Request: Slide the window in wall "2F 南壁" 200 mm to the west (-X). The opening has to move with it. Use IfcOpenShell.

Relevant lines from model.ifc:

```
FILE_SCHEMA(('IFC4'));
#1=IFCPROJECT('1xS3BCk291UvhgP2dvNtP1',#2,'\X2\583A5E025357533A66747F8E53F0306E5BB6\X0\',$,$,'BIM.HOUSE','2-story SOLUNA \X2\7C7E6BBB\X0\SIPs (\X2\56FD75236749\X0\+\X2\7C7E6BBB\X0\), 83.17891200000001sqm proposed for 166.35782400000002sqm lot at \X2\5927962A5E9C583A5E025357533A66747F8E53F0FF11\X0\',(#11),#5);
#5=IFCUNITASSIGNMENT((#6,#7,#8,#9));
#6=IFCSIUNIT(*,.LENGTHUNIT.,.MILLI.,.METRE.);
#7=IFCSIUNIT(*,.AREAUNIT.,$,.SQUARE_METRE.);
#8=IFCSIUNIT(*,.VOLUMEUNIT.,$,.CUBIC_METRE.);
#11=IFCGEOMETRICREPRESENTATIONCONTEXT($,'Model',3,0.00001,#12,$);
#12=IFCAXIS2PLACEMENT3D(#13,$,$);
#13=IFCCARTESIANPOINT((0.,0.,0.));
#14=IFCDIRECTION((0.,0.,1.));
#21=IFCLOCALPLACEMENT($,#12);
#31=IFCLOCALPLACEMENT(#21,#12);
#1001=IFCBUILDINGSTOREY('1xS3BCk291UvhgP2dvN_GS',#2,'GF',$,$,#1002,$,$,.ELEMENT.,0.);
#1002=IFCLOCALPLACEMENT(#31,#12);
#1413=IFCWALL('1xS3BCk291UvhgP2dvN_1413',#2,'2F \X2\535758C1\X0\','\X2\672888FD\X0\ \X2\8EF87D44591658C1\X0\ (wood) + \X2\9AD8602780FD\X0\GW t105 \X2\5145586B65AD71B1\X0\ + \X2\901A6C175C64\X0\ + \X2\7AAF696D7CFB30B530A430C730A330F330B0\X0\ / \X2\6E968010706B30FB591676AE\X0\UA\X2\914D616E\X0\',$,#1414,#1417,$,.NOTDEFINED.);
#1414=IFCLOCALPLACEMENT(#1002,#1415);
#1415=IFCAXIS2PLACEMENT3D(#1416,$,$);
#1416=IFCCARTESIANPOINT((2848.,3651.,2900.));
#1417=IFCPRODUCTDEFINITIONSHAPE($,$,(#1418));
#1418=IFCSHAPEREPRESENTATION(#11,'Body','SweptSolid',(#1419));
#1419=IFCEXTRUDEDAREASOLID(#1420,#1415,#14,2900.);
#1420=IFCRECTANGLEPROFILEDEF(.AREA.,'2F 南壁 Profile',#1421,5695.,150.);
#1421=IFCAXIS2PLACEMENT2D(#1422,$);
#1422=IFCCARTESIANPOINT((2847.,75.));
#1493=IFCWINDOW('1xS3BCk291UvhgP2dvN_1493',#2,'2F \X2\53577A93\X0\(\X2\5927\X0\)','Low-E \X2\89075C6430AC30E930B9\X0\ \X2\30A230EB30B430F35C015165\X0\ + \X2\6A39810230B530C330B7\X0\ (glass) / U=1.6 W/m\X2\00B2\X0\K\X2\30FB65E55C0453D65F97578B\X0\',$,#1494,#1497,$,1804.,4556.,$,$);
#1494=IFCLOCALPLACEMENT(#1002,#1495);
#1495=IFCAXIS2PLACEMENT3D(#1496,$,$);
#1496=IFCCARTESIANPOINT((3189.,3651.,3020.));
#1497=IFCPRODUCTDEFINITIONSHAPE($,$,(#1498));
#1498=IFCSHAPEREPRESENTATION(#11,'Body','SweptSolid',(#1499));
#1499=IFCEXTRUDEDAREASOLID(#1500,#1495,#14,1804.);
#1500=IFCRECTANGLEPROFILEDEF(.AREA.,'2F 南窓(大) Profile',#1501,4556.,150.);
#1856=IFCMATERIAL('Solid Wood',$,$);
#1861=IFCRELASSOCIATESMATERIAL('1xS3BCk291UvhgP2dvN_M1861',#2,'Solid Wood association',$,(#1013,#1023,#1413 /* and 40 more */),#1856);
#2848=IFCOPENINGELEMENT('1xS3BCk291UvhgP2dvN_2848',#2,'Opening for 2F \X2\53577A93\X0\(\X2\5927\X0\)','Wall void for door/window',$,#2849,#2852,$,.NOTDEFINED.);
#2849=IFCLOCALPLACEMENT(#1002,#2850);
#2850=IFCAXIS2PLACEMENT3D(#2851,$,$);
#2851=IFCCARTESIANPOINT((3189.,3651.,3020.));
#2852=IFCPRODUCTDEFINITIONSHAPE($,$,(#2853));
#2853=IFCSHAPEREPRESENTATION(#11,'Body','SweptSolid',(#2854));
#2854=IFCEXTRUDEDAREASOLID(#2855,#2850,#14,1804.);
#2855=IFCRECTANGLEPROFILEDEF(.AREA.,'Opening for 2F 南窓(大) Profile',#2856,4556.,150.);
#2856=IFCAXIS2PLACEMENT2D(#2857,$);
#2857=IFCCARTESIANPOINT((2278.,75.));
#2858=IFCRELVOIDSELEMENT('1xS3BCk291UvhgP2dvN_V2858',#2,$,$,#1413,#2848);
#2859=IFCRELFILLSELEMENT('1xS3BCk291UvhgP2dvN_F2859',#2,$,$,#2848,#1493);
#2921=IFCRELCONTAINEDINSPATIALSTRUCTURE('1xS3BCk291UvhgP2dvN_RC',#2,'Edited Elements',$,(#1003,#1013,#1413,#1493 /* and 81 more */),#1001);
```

```python
import ifcopenshell
import ifcopenshell.api.geometry
import ifcopenshell.util.placement

model = ifcopenshell.open("model.ifc")

window = model.by_guid("1xS3BCk291UvhgP2dvN_1493")
opening = window.FillsVoids[0].RelatingOpeningElement
wall = opening.VoidsElements[0].RelatingBuildingElement

wall_matrix = ifcopenshell.util.placement.get_local_placement(wall.ObjectPlacement)
shift = wall_matrix[:3, 0] * -200.0
before = ifcopenshell.util.placement.get_local_placement(window.ObjectPlacement)[:3, 3].copy()

# The window is not placed relative to its opening, so move both.
for product in (opening, window):
    matrix = ifcopenshell.util.placement.get_local_placement(product.ObjectPlacement)
    matrix[:3, 3] += shift
    ifcopenshell.api.geometry.edit_object_placement(model, product=product, matrix=matrix, is_si=False)

after = ifcopenshell.util.placement.get_local_placement(window.ObjectPlacement)[:3, 3]
print("window moved by", (after - before).round(3) + 0.0)

model.write("model_v2.ifc")
```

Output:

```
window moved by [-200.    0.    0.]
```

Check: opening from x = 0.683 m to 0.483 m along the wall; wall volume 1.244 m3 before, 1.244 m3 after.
